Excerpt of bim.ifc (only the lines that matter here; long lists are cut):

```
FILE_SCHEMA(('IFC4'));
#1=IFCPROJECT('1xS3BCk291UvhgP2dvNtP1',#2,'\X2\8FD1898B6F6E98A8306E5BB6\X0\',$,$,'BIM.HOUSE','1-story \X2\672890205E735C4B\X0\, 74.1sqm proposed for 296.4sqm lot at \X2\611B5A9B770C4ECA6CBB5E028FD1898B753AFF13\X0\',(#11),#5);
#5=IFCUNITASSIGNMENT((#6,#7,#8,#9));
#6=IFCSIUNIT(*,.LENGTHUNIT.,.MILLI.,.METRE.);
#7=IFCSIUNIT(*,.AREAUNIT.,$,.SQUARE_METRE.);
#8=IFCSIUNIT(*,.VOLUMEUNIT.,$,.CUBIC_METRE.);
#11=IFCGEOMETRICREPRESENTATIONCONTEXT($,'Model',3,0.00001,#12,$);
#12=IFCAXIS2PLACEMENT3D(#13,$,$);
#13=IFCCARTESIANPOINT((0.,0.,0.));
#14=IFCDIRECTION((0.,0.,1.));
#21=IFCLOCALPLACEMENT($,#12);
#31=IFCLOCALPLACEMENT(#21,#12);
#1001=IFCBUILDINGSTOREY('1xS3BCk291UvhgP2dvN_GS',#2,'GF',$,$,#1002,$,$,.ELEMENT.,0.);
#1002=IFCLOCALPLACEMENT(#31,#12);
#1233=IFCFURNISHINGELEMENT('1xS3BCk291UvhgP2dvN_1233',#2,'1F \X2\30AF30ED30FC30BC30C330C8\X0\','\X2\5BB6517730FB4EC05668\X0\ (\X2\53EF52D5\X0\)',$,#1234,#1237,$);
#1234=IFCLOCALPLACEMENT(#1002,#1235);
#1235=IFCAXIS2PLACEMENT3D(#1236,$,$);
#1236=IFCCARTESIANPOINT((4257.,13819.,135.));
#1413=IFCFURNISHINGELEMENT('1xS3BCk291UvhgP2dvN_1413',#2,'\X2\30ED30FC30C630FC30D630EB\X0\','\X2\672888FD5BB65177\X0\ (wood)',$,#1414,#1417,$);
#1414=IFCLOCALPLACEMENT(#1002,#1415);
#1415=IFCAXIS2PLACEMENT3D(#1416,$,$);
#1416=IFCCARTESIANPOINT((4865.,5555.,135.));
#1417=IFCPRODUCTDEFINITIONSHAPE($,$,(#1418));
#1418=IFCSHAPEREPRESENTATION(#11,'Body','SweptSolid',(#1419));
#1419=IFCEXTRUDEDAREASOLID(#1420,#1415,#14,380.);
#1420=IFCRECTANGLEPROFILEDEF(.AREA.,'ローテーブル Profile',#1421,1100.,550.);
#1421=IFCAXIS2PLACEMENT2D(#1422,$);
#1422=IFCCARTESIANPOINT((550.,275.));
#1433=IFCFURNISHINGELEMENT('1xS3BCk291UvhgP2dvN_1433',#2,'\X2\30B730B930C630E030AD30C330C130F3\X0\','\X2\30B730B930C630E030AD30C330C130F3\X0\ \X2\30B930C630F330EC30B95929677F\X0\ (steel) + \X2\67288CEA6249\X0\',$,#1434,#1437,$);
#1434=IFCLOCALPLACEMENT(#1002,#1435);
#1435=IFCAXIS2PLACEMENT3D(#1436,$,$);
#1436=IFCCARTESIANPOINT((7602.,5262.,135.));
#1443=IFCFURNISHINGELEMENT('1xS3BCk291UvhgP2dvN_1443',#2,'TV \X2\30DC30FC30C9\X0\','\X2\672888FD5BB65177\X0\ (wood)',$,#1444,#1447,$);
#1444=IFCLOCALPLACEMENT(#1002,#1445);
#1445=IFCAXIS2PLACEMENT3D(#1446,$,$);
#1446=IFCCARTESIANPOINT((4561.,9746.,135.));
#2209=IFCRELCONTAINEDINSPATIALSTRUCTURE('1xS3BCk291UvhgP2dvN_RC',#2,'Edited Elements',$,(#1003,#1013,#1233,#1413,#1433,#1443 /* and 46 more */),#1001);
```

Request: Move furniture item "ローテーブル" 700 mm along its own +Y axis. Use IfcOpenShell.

```python
import ifcopenshell
import ifcopenshell.api.geometry
import ifcopenshell.util.placement
import ifcopenshell.util.unit

model = ifcopenshell.open("bim.ifc")
unit_scale = ifcopenshell.util.unit.calculate_unit_scale(model)

item = model.by_guid("1xS3BCk291UvhgP2dvN_1413")
matrix = ifcopenshell.util.placement.get_local_placement(item.ObjectPlacement)
matrix[:3, 3] += matrix[:3, 1] * 0.7 / unit_scale
ifcopenshell.api.geometry.edit_object_placement(model, product=item, matrix=matrix, is_si=False)

print(ifcopenshell.util.placement.get_local_placement(item.ObjectPlacement).round(3) + 0.0)

model.write("bim_v2.ifc")
```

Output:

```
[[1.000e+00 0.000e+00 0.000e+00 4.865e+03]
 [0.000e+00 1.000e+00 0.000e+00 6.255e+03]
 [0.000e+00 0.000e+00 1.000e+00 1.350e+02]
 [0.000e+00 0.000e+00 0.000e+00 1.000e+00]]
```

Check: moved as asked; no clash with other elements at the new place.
